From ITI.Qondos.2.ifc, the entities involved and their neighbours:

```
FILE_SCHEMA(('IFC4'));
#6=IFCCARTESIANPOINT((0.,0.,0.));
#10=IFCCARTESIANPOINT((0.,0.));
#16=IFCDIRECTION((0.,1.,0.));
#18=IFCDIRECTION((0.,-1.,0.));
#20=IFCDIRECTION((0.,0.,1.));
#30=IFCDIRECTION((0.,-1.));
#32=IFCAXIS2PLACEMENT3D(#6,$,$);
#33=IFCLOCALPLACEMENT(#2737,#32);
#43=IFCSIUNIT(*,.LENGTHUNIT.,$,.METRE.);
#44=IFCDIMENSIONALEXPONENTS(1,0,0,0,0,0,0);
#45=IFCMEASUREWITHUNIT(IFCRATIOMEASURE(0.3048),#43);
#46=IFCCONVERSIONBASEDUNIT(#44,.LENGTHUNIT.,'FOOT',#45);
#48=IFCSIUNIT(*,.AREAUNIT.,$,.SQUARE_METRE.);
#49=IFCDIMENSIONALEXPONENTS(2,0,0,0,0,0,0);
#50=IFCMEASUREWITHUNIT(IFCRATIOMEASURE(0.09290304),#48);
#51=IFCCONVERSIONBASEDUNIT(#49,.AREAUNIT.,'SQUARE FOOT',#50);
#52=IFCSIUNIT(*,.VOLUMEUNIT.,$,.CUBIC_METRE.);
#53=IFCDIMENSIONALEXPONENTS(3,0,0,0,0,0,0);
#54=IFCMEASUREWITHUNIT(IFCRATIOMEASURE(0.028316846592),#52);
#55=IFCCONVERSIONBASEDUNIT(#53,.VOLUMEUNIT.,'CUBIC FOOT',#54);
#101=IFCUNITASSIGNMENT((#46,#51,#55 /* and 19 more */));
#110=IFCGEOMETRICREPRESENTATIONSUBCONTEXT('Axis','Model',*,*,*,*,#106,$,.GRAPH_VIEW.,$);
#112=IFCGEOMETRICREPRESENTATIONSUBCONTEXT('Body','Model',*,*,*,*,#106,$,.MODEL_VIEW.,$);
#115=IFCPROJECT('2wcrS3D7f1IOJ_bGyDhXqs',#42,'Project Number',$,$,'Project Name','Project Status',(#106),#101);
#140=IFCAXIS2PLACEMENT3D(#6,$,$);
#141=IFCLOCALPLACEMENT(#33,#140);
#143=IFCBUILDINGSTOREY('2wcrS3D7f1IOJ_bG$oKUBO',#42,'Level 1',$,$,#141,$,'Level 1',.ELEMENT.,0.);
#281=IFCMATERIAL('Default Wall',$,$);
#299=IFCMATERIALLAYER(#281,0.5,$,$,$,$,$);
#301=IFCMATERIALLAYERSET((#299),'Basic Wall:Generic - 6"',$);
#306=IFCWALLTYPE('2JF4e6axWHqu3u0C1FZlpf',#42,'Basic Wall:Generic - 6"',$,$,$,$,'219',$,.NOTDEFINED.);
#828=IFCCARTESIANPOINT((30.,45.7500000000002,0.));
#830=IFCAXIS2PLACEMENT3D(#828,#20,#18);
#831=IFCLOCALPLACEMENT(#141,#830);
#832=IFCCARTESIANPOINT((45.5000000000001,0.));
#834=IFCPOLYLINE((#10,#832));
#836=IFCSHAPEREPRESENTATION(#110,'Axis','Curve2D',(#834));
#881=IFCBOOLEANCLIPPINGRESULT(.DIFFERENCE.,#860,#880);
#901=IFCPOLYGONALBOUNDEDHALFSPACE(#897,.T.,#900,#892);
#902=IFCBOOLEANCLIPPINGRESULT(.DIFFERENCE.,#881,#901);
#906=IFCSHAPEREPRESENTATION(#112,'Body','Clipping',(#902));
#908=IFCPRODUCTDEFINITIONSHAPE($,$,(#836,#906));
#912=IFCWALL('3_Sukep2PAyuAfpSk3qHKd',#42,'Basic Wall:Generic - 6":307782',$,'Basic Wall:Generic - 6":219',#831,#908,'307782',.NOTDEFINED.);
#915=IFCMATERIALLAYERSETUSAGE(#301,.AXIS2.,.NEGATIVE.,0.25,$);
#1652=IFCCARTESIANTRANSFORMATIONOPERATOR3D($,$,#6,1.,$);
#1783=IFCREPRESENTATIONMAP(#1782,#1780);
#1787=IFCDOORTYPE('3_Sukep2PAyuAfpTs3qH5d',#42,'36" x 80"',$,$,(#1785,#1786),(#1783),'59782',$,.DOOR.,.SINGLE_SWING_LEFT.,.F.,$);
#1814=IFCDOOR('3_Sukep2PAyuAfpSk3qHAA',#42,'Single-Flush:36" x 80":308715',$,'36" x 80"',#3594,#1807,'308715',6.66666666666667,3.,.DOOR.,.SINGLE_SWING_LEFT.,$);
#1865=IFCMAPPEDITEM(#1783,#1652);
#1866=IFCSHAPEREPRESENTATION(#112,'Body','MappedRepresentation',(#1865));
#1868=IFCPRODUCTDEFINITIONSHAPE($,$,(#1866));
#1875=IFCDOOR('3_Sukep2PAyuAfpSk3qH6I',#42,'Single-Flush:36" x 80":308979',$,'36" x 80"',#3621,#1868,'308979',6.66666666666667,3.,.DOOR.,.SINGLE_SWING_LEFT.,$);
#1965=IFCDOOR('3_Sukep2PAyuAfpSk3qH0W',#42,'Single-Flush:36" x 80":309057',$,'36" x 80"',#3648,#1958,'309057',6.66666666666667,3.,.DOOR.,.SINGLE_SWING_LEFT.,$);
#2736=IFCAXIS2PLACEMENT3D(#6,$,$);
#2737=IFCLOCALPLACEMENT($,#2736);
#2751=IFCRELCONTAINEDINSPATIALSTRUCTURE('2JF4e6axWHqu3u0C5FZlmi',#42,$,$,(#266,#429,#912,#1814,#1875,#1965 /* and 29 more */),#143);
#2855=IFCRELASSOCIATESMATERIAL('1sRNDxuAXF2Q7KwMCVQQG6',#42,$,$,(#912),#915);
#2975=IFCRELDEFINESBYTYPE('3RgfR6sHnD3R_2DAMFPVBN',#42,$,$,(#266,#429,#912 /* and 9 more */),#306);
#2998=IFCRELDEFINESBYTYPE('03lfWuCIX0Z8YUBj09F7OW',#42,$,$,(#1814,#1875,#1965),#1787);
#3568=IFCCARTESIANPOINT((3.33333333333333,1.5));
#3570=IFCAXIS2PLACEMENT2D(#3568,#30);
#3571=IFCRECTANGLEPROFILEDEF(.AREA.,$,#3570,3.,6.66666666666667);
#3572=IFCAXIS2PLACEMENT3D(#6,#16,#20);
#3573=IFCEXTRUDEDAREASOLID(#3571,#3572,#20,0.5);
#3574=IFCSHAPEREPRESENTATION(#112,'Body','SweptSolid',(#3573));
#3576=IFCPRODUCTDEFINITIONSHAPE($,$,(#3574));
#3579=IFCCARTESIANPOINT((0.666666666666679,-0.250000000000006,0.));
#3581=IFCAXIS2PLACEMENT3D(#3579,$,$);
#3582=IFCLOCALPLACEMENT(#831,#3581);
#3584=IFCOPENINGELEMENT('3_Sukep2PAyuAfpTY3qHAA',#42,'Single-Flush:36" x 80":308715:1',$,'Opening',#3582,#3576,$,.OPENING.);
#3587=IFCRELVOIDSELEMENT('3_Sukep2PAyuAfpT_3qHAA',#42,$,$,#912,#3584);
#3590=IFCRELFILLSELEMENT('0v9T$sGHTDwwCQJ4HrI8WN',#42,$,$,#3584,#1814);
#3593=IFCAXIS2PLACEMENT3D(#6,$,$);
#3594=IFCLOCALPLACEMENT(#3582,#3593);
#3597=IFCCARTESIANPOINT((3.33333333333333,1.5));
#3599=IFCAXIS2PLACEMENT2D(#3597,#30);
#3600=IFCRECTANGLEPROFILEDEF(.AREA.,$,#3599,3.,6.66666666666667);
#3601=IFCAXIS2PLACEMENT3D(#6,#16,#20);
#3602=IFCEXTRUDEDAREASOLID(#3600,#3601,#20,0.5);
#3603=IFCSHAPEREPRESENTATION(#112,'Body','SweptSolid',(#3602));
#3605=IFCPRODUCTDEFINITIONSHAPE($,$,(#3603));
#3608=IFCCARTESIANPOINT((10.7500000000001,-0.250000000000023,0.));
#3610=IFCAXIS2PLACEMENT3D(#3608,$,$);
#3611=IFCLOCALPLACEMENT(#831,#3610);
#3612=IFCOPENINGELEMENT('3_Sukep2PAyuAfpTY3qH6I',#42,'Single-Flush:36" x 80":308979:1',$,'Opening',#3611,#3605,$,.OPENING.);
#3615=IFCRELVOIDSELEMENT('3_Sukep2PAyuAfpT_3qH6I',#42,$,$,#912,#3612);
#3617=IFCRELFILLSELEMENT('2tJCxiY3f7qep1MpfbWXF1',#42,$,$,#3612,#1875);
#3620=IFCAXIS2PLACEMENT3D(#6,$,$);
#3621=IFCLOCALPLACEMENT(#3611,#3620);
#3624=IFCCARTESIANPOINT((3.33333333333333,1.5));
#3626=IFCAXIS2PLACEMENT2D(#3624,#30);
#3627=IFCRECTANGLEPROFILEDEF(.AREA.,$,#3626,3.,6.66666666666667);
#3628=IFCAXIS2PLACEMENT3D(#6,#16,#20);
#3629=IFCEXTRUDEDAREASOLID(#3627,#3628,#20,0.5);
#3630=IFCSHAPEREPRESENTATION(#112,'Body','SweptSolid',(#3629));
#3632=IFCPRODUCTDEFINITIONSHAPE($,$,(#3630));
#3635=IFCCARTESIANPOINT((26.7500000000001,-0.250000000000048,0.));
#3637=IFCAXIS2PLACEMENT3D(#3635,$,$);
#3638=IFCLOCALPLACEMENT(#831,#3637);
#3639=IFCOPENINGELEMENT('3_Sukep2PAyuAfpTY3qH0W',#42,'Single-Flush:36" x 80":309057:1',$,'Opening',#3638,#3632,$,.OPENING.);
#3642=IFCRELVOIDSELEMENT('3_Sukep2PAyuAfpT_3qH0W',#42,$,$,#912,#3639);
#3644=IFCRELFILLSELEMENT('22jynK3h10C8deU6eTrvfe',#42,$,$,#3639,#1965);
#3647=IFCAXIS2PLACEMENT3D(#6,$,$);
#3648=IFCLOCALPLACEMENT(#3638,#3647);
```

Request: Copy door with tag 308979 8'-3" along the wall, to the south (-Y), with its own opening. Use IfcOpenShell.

```python
import ifcopenshell
import ifcopenshell.api.feature
import ifcopenshell.api.geometry
import ifcopenshell.api.root
import ifcopenshell.geom
import ifcopenshell.util.element
import ifcopenshell.util.placement
import ifcopenshell.util.shape
import ifcopenshell.util.unit

model = ifcopenshell.open("ITI.Qondos.2.ifc")
unit_scale = ifcopenshell.util.unit.calculate_unit_scale(model)
settings = ifcopenshell.geom.settings()


def volume(element):
    """Net volume in cubic metres, openings subtracted."""
    shape = ifcopenshell.geom.create_shape(settings, element)
    return ifcopenshell.util.shape.get_volume(shape.geometry)


def reuse_history(source, copy):
    """copy_class also copies each property set's owner history, people and application; keep the originals."""
    for rel in copy.IsDefinedBy:
        if rel.is_a("IfcRelDefinesByProperties") and (history := rel.RelatingPropertyDefinition.OwnerHistory):
            rel.RelatingPropertyDefinition.OwnerHistory = source.OwnerHistory
            ifcopenshell.util.element.remove_deep2(model, history)


door = model.by_guid("3_Sukep2PAyuAfpSk3qH6I")
opening = door.FillsVoids[0].RelatingOpeningElement
wall = opening.VoidsElements[0].RelatingBuildingElement
before = volume(wall)
shift = ifcopenshell.util.placement.get_local_placement(wall.ObjectPlacement)[:3, 0] * 99 * 0.0254 / unit_scale

# copy_class copies the void relationship, type, container and properties, but no geometry.
new_opening = ifcopenshell.api.root.copy_class(model, product=opening)
new_opening.Representation = ifcopenshell.util.element.copy_deep(
    model, opening.Representation, exclude=["IfcGeometricRepresentationContext", "IfcRepresentationMap"]
)
new_opening.Name = 'Single-Flush:36" x 80"'
new_door = ifcopenshell.api.root.copy_class(model, product=door)
new_door.Representation = ifcopenshell.util.element.copy_deep(
    model, door.Representation, exclude=["IfcGeometricRepresentationContext", "IfcRepresentationMap"]
)
new_door.Name = 'Single-Flush:36" x 80"'
new_door.Tag = None
reuse_history(door, new_door)
ifcopenshell.api.feature.add_filling(model, opening=new_opening, element=new_door)

for old, new in ((opening, new_opening), (door, new_door)):
    matrix = ifcopenshell.util.placement.get_local_placement(old.ObjectPlacement)
    matrix[:3, 3] += shift
    ifcopenshell.api.geometry.edit_object_placement(model, product=new, matrix=matrix, is_si=False)

after = volume(wall)

print(f"wall volume {before:.3f} -> {after:.3f} m3")

model.write("ITI.Qondos.2_updated.ifc")
```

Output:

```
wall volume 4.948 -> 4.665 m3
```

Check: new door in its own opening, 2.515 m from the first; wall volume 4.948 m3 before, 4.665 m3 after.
